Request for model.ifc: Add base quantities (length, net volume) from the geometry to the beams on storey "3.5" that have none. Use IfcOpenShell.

First a look at what the model holds.

```python
import ifcopenshell
import ifcopenshell.util.element
import ifcopenshell.util.unit

model = ifcopenshell.open("model.ifc")
print(model.schema)
for unit_type in ("LENGTHUNIT", "AREAUNIT", "VOLUMEUNIT"):
    print(unit_type, ifcopenshell.util.unit.calculate_unit_scale(model, unit_type))
storey = next(s for s in model.by_type("IfcBuildingStorey") if s.Name == "3.5")
beams = [e for e in ifcopenshell.util.element.get_decomposition(storey) if e.is_a("IfcBeam")]
for e in sorted(beams, key=lambda e: e.id()):
    print(e.id(), e.is_a(), e.Name, list(ifcopenshell.util.element.get_psets(e, qtos_only=True)), sep=" | ")
```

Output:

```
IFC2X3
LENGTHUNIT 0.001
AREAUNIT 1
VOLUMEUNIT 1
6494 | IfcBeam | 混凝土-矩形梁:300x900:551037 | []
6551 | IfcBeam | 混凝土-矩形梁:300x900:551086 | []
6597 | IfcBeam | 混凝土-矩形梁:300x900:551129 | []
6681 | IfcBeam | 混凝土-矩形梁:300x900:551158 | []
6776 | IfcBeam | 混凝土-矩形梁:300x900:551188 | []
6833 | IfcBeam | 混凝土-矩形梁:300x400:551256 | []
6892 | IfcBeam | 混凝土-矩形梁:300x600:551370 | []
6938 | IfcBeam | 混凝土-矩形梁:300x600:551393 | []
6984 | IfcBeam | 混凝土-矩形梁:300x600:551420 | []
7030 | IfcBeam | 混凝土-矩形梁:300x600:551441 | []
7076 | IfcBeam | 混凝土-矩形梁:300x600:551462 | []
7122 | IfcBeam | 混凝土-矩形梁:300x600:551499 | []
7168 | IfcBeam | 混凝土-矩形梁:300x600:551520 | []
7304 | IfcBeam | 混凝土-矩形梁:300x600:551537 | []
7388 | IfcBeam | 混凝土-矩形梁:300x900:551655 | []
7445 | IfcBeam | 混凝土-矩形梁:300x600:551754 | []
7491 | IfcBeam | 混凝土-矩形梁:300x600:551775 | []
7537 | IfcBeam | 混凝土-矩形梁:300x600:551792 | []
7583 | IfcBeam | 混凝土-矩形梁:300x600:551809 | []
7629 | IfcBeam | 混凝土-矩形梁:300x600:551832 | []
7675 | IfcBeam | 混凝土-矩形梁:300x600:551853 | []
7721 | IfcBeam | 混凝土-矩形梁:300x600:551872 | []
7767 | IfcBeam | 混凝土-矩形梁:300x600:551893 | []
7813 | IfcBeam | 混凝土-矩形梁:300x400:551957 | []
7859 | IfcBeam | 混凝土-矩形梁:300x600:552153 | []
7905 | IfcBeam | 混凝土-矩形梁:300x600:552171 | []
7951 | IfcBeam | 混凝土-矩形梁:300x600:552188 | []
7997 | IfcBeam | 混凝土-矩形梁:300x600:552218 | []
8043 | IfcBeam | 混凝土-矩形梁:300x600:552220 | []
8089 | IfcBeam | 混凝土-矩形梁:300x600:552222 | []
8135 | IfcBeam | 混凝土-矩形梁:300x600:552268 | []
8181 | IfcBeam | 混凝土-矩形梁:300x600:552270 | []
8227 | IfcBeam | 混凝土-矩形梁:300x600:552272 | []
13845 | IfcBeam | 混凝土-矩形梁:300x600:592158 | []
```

```python
import ifcopenshell
import ifcopenshell.api.pset
import ifcopenshell.geom
import ifcopenshell.util.element
import ifcopenshell.util.shape
import ifcopenshell.util.unit

model = ifcopenshell.open("model.ifc")
unit_scale = ifcopenshell.util.unit.calculate_unit_scale(model)
volume_scale = ifcopenshell.util.unit.calculate_unit_scale(model, "VOLUMEUNIT")
settings = ifcopenshell.geom.settings()

storey = next(s for s in model.by_type("IfcBuildingStorey") if s.Name == "3.5")
beams = [e for e in ifcopenshell.util.element.get_decomposition(storey) if e.is_a("IfcBeam")]

for e in sorted(beams, key=lambda e: e.id()):
    if ifcopenshell.util.element.get_psets(e, qtos_only=True, should_inherit=False):
        continue
    # Geometry comes back in metres, in the element's own axes.
    shape = ifcopenshell.geom.create_shape(settings, e)
    values = {
        "Length": ifcopenshell.util.shape.get_max_xyz(shape.geometry) / unit_scale,
        "NetVolume": ifcopenshell.util.shape.get_volume(shape.geometry) / volume_scale,
    }
    qto = ifcopenshell.api.pset.add_qto(model, product=e, name="BaseQuantities")
    ifcopenshell.api.pset.edit_qto(model, qto=qto, properties=values)
    print(e.id(), {k: round(v, 3) for k, v in values.items()})

model.write("model_v2.ifc")
```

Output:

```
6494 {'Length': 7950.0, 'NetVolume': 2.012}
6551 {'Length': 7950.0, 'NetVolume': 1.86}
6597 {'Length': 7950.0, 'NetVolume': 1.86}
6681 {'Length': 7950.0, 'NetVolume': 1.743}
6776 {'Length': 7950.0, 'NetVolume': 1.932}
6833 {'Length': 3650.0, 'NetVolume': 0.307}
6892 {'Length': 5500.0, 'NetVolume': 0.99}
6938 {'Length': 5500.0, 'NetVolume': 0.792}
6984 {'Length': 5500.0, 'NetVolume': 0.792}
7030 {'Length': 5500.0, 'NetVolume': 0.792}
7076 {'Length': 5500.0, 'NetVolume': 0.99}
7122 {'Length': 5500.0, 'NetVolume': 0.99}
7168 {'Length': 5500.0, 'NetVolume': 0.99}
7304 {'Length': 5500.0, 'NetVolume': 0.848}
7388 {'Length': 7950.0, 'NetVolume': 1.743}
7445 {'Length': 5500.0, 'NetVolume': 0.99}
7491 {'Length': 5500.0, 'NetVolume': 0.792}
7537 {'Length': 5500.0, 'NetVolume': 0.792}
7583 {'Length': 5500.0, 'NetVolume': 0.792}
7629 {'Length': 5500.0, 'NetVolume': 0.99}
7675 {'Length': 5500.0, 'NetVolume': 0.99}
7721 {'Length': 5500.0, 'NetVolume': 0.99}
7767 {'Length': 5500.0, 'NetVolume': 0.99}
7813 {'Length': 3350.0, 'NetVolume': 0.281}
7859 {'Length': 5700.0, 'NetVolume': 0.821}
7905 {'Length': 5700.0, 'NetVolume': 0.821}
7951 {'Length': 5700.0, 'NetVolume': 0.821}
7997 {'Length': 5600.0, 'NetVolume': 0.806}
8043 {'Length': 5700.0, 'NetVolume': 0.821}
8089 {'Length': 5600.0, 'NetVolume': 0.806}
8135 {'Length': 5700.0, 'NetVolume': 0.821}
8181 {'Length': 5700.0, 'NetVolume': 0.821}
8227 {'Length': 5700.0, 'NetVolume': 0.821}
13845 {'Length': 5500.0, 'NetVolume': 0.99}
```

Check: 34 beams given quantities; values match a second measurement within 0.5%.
